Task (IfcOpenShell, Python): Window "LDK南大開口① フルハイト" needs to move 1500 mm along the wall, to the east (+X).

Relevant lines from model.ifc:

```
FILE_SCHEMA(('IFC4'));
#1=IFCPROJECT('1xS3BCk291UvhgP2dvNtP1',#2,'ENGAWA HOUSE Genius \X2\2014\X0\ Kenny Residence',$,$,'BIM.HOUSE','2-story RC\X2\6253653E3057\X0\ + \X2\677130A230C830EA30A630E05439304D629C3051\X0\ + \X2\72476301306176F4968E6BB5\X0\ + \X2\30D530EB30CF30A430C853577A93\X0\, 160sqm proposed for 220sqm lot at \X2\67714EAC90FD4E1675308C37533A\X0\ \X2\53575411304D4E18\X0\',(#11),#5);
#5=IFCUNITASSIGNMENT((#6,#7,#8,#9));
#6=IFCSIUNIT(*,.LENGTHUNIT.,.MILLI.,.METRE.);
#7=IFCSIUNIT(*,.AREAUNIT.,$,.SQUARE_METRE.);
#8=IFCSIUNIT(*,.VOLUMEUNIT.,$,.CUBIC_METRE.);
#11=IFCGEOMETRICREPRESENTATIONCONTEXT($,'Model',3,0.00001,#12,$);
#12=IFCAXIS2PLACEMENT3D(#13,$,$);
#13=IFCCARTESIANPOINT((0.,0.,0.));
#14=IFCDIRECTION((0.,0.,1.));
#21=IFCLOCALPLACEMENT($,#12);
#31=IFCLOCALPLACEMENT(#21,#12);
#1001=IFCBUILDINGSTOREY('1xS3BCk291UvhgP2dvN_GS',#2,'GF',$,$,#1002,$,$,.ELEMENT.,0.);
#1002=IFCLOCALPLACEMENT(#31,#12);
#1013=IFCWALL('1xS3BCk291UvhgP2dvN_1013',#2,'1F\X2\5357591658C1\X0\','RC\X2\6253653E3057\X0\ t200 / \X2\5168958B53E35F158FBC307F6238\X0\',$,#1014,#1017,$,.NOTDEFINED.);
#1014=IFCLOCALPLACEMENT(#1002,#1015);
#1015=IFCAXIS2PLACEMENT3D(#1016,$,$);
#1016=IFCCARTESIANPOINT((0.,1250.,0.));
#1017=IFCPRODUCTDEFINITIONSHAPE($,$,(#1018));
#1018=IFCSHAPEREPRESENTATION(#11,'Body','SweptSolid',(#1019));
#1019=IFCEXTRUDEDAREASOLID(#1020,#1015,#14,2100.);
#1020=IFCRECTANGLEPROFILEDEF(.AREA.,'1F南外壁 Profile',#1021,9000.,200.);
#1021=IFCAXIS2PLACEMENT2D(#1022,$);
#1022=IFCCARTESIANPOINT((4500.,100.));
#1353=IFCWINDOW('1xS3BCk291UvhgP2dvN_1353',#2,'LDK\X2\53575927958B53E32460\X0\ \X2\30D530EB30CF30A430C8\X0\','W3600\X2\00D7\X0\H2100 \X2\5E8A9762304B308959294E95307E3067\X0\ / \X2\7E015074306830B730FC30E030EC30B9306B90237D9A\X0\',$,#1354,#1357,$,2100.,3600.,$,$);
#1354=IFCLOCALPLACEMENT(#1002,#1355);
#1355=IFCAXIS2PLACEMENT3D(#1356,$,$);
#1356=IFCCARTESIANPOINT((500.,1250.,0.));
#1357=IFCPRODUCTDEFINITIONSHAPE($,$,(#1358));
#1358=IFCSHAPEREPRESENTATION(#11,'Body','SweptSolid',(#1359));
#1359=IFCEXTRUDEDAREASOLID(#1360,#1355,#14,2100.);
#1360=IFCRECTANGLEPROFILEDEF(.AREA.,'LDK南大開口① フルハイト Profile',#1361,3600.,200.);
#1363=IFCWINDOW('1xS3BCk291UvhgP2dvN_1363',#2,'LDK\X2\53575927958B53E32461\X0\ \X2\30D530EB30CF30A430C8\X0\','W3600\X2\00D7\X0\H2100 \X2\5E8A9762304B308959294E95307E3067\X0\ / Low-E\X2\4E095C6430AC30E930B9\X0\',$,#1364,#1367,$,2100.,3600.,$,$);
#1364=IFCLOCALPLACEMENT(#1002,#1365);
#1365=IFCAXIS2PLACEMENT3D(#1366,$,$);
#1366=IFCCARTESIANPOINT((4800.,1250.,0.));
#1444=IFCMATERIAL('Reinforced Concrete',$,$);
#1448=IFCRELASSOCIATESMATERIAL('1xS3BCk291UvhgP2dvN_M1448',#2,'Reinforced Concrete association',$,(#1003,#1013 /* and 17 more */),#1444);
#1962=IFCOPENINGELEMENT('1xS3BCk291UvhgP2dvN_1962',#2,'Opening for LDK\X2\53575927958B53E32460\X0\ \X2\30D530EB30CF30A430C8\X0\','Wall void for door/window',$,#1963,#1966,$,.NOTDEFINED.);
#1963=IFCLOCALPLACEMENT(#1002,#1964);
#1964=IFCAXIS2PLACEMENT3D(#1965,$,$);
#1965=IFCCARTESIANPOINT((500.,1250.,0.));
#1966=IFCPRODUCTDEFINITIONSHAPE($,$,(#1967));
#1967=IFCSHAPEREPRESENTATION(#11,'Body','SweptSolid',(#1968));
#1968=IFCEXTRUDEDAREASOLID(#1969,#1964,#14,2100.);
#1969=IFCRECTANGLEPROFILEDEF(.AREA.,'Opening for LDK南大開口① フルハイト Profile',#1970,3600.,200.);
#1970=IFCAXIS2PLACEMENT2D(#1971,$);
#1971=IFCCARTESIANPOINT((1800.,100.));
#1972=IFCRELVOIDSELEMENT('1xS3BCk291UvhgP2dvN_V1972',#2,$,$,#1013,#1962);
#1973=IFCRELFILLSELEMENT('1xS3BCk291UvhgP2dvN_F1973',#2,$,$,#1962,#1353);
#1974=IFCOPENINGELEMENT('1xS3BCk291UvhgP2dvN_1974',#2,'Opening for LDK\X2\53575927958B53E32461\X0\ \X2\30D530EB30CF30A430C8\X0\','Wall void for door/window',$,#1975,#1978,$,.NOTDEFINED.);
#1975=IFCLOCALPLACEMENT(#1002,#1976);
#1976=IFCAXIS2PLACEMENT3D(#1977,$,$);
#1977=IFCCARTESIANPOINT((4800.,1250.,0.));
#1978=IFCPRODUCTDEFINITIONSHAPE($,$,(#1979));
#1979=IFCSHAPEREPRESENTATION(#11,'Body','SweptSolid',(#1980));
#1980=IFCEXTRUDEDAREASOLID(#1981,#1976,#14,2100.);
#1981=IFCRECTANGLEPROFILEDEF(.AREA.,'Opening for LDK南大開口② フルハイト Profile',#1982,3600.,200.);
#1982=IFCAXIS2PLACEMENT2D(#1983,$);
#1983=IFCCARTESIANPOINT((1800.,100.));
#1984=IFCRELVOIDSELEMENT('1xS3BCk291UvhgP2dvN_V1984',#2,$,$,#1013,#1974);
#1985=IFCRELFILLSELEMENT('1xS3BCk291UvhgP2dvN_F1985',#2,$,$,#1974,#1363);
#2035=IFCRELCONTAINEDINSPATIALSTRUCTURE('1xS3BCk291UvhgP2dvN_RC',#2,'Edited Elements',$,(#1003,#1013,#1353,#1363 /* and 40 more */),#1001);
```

```python
import ifcopenshell
import ifcopenshell.api.geometry
import ifcopenshell.util.placement

model = ifcopenshell.open("model.ifc")

window = model.by_guid("1xS3BCk291UvhgP2dvN_1353")
opening = window.FillsVoids[0].RelatingOpeningElement
wall = opening.VoidsElements[0].RelatingBuildingElement

wall_matrix = ifcopenshell.util.placement.get_local_placement(wall.ObjectPlacement)
shift = wall_matrix[:3, 0] * 1500.0
before = ifcopenshell.util.placement.get_local_placement(window.ObjectPlacement)[:3, 3].copy()

# The window is not placed relative to its opening, so move both.
for product in (opening, window):
    matrix = ifcopenshell.util.placement.get_local_placement(product.ObjectPlacement)
    matrix[:3, 3] += shift
    ifcopenshell.api.geometry.edit_object_placement(model, product=product, matrix=matrix, is_si=False)

after = ifcopenshell.util.placement.get_local_placement(window.ObjectPlacement)[:3, 3]
print("window moved by", (after - before).round(3) + 0.0)

model.write("model_rev.ifc")
```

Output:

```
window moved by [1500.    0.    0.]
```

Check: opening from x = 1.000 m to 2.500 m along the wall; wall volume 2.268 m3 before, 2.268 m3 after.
